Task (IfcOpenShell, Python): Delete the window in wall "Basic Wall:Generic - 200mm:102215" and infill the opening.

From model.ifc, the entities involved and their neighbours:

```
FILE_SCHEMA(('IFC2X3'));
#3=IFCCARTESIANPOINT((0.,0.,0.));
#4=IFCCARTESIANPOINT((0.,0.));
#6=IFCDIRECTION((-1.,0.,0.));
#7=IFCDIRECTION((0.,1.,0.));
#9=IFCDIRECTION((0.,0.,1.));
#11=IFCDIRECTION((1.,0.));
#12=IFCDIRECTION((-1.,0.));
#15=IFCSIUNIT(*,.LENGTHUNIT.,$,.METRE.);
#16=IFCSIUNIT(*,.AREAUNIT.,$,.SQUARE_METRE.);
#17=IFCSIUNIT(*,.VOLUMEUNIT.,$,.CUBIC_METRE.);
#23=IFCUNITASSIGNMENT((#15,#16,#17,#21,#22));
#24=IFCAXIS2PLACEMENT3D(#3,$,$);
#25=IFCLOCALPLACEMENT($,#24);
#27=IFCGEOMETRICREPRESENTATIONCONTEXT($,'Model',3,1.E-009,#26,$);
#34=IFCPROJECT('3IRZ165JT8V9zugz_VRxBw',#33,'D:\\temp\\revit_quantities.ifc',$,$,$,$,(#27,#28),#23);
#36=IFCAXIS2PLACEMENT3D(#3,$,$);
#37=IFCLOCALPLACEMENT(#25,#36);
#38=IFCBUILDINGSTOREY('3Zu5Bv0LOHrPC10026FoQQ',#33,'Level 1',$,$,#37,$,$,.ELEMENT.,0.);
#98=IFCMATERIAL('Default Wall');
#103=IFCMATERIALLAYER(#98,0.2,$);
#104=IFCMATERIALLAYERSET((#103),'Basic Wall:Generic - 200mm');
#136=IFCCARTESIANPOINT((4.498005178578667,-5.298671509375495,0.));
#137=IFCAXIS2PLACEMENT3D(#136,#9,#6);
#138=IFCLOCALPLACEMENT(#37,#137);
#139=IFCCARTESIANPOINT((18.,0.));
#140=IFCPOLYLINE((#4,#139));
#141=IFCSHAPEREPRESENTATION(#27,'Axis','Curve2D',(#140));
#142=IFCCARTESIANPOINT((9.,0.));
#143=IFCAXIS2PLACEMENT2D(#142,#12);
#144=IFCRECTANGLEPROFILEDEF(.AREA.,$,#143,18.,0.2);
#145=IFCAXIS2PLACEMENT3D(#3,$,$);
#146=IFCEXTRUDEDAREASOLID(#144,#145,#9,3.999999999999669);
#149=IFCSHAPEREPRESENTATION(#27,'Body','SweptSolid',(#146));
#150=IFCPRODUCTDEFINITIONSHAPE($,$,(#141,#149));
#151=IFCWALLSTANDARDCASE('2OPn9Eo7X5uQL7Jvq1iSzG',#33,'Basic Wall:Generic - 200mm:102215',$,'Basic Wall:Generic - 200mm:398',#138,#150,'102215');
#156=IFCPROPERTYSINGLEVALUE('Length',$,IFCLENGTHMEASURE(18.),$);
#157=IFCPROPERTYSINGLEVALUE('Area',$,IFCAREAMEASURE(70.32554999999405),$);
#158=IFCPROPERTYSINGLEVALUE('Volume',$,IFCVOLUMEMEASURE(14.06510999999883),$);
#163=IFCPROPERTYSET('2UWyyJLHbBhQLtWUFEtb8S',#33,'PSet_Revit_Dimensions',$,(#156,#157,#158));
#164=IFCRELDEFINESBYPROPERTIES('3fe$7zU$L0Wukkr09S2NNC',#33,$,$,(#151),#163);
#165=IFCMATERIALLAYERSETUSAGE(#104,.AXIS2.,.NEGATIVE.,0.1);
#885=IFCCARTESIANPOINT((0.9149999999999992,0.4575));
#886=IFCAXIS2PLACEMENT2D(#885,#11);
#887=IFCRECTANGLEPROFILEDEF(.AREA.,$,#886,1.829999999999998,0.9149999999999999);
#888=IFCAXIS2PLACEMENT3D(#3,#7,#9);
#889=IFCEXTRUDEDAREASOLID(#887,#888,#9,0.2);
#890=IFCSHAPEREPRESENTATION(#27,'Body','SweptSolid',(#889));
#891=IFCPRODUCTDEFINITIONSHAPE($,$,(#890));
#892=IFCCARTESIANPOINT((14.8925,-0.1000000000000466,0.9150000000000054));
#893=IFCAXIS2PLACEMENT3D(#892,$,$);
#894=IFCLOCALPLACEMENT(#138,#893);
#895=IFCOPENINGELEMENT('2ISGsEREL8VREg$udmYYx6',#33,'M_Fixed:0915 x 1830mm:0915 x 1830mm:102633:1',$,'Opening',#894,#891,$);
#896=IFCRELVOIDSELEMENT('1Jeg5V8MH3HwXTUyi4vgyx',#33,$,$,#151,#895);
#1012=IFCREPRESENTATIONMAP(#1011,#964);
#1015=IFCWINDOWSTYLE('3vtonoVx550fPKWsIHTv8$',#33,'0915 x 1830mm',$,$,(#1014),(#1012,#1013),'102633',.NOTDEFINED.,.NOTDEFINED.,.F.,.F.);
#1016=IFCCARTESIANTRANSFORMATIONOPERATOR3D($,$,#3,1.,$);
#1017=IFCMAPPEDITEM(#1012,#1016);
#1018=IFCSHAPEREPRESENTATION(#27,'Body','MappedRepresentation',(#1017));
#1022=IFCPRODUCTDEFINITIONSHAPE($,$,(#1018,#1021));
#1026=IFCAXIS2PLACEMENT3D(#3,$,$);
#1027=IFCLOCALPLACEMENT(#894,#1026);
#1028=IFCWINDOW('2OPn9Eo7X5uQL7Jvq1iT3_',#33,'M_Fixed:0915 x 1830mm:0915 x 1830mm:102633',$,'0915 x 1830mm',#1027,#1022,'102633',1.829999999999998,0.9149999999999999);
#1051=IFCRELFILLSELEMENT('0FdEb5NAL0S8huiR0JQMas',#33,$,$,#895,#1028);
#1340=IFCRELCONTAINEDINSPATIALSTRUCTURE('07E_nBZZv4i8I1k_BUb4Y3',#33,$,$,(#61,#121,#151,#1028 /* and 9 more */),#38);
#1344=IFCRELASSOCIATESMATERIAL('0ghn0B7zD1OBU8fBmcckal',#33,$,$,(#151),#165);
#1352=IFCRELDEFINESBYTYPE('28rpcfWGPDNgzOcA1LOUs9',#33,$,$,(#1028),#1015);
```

```python
import ifcopenshell
import ifcopenshell.api.feature
import ifcopenshell.api.pset
import ifcopenshell.api.root
import ifcopenshell.geom
import ifcopenshell.util.element
import ifcopenshell.util.shape
import ifcopenshell.util.unit

model = ifcopenshell.open("model.ifc")
area_scale = ifcopenshell.util.unit.calculate_unit_scale(model, "AREAUNIT")
volume_scale = ifcopenshell.util.unit.calculate_unit_scale(model, "VOLUMEUNIT")
settings = ifcopenshell.geom.settings()


def volume(element):
    """Net volume in cubic metres, openings subtracted."""
    shape = ifcopenshell.geom.create_shape(settings, element)
    return ifcopenshell.util.shape.get_volume(shape.geometry)


window = model.by_guid("2OPn9Eo7X5uQL7Jvq1iT3_")
opening = window.FillsVoids[0].RelatingOpeningElement
wall = opening.VoidsElements[0].RelatingBuildingElement
before = volume(wall)

ifcopenshell.api.root.remove_product(model, product=window)
ifcopenshell.api.feature.remove_feature(model, feature=opening)

after = volume(wall)
thickness = 0.2  # wall thickness in metres

# Update the wall's stored quantities.
pset = model.by_id(ifcopenshell.util.element.get_pset(wall, "PSet_Revit_Dimensions", should_inherit=False)["id"])
ifcopenshell.api.pset.edit_pset(model, pset=pset, properties={
    "Area": model.create_entity("IfcAreaMeasure", after / thickness / area_scale),
    "Volume": model.create_entity("IfcVolumeMeasure", after / volume_scale),
})

print(f"wall volume {before:.3f} -> {after:.3f} m3")

model.write("model_v2.ifc")
```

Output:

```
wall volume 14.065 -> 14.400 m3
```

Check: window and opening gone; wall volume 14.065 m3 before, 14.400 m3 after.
